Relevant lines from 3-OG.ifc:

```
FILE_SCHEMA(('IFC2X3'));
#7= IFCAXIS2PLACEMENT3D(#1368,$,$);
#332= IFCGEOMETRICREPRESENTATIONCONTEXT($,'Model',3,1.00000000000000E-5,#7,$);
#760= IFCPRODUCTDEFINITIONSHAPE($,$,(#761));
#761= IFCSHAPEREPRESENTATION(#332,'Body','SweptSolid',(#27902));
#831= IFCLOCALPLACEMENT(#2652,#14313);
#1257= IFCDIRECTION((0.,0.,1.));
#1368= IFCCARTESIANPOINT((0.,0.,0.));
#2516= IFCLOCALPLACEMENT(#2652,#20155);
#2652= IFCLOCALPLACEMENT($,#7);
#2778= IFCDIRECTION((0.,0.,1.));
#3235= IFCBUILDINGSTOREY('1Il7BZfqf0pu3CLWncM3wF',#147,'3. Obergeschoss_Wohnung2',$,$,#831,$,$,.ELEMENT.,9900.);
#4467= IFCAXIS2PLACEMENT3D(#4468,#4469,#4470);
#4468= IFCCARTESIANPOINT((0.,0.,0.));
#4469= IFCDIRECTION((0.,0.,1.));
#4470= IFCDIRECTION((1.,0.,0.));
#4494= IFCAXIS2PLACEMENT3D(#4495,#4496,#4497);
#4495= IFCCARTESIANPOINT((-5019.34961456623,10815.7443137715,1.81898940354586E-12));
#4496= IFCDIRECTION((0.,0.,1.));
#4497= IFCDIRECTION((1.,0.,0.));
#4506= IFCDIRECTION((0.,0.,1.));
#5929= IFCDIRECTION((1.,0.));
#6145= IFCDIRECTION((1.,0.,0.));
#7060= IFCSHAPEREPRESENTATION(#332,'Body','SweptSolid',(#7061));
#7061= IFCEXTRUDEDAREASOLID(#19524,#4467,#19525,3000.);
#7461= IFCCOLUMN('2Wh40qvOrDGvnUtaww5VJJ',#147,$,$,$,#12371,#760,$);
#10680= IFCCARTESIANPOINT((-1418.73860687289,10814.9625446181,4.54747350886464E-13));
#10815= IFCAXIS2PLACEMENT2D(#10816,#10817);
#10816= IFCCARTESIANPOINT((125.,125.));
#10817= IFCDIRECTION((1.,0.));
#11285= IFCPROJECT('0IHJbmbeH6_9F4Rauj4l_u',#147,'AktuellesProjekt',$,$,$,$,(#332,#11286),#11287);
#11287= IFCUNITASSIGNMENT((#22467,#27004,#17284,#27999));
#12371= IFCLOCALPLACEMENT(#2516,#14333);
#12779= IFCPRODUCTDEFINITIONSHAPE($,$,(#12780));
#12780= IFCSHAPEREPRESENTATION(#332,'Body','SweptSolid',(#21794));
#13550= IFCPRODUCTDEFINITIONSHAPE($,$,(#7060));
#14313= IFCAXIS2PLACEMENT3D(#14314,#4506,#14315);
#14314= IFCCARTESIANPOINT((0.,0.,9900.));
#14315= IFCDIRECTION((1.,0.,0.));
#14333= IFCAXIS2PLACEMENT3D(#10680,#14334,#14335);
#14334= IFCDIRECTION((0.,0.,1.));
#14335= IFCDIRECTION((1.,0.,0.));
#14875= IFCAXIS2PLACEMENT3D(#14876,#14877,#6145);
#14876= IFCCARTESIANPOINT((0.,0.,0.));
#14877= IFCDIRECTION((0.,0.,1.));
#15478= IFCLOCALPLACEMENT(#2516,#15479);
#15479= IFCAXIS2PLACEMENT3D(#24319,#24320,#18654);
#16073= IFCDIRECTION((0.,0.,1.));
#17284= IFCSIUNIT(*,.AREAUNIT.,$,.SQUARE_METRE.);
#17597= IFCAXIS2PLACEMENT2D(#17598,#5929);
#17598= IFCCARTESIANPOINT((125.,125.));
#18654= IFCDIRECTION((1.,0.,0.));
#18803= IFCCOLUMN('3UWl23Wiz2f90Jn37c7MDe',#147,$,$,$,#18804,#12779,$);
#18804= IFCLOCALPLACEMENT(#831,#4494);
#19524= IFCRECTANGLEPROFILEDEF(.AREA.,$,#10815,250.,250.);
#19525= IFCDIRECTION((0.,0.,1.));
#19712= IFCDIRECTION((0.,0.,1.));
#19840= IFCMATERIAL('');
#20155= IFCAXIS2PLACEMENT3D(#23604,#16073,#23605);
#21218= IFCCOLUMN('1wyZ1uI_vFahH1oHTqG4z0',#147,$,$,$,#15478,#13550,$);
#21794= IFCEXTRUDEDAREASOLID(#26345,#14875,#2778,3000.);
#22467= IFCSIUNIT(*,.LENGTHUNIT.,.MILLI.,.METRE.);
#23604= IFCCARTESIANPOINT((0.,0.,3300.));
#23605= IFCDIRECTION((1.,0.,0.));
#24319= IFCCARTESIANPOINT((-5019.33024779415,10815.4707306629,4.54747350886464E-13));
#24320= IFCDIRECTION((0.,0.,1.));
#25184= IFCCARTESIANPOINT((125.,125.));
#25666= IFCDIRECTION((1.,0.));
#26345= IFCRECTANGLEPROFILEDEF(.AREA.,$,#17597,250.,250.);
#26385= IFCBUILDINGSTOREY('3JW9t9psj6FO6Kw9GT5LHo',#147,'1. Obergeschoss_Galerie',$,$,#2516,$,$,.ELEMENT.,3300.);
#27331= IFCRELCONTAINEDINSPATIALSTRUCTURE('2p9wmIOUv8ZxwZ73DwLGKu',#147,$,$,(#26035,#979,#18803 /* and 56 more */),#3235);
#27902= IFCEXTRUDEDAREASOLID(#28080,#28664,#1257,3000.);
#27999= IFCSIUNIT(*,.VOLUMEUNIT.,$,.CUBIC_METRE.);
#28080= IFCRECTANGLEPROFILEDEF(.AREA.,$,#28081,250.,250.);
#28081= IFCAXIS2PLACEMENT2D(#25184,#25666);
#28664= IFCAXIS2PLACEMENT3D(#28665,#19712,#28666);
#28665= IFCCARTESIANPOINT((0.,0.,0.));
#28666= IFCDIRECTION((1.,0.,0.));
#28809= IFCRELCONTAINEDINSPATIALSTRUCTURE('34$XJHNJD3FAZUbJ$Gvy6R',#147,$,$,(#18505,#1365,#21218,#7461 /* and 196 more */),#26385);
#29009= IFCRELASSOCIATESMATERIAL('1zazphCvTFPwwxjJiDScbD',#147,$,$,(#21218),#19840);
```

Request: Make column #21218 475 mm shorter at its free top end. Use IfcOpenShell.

```python
import ifcopenshell
import ifcopenshell.util.unit

model = ifcopenshell.open("3-OG.ifc")
unit_scale = ifcopenshell.util.unit.calculate_unit_scale(model)

member = model.by_id(21218)
change = -0.475 / unit_scale

# The extrusion runs towards the end named, so only its depth changes.
body = next(r for r in member.Representation.Representations if r.RepresentationIdentifier == "Body")
solid = body.Items[0]
old_length = solid.Depth
solid.Depth += change

print(f"length {old_length:g} -> {solid.Depth:g}")

model.write("3-OG_v2.ifc")
```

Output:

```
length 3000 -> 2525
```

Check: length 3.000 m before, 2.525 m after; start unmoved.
